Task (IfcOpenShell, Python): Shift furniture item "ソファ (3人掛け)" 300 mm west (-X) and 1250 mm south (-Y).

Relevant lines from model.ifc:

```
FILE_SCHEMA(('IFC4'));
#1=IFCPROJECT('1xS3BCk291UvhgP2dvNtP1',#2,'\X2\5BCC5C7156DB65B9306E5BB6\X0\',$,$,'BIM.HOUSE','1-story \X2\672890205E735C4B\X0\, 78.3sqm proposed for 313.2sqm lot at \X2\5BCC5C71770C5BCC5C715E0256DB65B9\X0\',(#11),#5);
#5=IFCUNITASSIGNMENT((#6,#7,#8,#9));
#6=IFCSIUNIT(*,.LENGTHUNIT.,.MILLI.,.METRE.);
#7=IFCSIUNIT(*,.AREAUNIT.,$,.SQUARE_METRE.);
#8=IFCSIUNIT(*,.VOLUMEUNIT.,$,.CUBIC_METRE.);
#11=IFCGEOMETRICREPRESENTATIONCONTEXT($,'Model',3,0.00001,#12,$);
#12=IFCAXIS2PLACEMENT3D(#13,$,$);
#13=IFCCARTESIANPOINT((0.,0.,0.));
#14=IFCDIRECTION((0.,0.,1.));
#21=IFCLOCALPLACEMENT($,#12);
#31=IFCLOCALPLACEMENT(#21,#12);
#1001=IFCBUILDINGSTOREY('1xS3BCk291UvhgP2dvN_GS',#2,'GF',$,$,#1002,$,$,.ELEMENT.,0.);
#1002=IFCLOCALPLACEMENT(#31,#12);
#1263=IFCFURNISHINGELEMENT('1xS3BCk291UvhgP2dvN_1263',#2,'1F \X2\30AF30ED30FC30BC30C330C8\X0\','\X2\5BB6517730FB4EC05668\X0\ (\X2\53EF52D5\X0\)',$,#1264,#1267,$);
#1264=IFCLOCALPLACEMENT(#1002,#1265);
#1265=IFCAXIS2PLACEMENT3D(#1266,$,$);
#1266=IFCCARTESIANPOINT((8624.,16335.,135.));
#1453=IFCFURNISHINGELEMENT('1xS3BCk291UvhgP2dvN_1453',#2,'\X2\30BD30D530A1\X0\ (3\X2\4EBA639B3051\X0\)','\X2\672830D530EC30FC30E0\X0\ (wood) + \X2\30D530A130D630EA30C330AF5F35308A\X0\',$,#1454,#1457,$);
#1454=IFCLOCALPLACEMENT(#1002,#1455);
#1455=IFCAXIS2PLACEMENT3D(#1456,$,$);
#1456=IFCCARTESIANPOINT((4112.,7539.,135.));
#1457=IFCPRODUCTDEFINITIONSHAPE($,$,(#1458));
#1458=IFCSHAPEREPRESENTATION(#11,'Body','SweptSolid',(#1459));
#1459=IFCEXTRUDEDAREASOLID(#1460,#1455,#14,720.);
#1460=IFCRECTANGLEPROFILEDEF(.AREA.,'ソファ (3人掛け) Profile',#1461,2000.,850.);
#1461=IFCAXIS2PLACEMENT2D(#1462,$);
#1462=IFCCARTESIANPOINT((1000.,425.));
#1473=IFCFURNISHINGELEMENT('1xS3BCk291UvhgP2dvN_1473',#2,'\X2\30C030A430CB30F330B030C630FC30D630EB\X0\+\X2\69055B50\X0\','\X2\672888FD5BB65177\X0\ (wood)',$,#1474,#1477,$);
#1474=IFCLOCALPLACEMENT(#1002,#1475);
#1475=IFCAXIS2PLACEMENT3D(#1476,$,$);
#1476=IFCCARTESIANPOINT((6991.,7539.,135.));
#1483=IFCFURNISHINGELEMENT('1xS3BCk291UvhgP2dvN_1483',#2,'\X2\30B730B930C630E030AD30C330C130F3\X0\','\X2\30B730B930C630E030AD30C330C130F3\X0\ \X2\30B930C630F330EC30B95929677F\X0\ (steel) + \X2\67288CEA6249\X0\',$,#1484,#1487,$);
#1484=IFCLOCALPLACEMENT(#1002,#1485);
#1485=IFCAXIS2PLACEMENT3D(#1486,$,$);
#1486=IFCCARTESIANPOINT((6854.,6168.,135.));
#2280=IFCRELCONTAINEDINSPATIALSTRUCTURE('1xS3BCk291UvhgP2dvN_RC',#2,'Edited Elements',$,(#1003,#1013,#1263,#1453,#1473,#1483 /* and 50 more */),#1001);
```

```python
import ifcopenshell
import ifcopenshell.api.geometry
import ifcopenshell.util.placement
import ifcopenshell.util.unit

model = ifcopenshell.open("model.ifc")
unit_scale = ifcopenshell.util.unit.calculate_unit_scale(model)

item = model.by_id(1453)
matrix = ifcopenshell.util.placement.get_local_placement(item.ObjectPlacement)
matrix[0, 3] -= 0.3 / unit_scale
matrix[1, 3] -= 1.25 / unit_scale
ifcopenshell.api.geometry.edit_object_placement(model, product=item, matrix=matrix, is_si=False)

print(ifcopenshell.util.placement.get_local_placement(item.ObjectPlacement).round(3) + 0.0)

model.write("model-out.ifc")
```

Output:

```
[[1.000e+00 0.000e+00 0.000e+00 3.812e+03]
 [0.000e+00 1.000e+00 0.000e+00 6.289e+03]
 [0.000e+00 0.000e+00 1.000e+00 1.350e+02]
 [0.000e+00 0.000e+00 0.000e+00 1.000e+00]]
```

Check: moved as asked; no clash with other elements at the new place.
